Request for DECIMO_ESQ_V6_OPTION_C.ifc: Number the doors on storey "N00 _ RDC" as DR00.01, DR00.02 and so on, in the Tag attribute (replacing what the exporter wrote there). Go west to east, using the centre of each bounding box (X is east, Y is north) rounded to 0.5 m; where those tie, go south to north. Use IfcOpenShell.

First a look at what the model holds.

```python
import ifcopenshell
import ifcopenshell.util.element
import ifcopenshell.util.placement

model = ifcopenshell.open("DECIMO_ESQ_V6_OPTION_C.ifc")
print(model.schema)
storey = next(s for s in model.by_type("IfcBuildingStorey") if s.Name == "N00 _ RDC")
doors = [e for e in ifcopenshell.util.element.get_decomposition(storey) if e.is_a("IfcDoor")]
for e in sorted(doors, key=lambda e: e.id()):
    origin = ifcopenshell.util.placement.get_local_placement(e.ObjectPlacement)[:3, 3]
    print(e.id(), e.Tag, e.Name, origin.round(2) + 0.0, sep=" | ")
```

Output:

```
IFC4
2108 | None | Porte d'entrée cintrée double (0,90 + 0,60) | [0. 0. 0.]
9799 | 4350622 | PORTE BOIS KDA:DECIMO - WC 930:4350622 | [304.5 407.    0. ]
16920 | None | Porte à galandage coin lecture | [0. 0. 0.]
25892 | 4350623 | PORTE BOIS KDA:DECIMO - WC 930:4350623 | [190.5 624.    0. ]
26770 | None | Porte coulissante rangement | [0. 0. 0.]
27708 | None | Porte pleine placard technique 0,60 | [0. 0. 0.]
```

```python
import ifcopenshell
import ifcopenshell.geom
import ifcopenshell.util.element
import ifcopenshell.util.shape

model = ifcopenshell.open("DECIMO_ESQ_V6_OPTION_C.ifc")
settings = ifcopenshell.geom.settings()
settings.set("use-world-coords", True)


def centre(element):
    shape = ifcopenshell.geom.create_shape(settings, element)
    return ifcopenshell.util.shape.get_bbox_centroid(shape.geometry)


storey = next(s for s in model.by_type("IfcBuildingStorey") if s.Name == "N00 _ RDC")
doors = [e for e in ifcopenshell.util.element.get_decomposition(storey) if e.is_a("IfcDoor")]

# Insertion points can sit at a corner or the storey origin, so sort by the geometry (in metres).
centres = {e: centre(e) for e in doors}
doors.sort(key=lambda e: (round(centres[e][0] / 0.5), centres[e][1]))

for i, e in enumerate(doors, start=1):
    number = f"DR00.{i:02d}"
    e.Tag = number
    print(e.id(), number)

model.write("DECIMO_ESQ_V6_OPTION_C_v2.ifc")
```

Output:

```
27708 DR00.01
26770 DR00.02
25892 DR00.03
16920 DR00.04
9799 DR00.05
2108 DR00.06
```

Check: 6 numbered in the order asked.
